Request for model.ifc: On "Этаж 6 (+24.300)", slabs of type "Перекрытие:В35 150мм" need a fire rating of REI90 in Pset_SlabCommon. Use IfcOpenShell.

First a look at what the model holds.

```python
import ifcopenshell
import ifcopenshell.util.element

model = ifcopenshell.open("model.ifc")
print(model.schema)
storey = next(s for s in model.by_type("IfcBuildingStorey") if s.Name == "Этаж 6 (+24.300)")
slabs = [e for e in ifcopenshell.util.element.get_decomposition(storey) if e.is_a("IfcSlab")]
seen = {}
for e in slabs:
    element_type = ifcopenshell.util.element.get_type(e)
    key = (element_type.Name if element_type != e and element_type else None, ifcopenshell.util.element.get_pset(e, "Pset_SlabCommon", "FireRating"))
    seen[key] = seen.get(key, 0) + 1
for (name, value), count in sorted(seen.items(), key=str):
    print(count, "x", name, "|", value)
```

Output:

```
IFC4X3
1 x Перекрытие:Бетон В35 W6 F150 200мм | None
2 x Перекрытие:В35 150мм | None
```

```python
import ifcopenshell
import ifcopenshell.api.pset
import ifcopenshell.util.element

model = ifcopenshell.open("model.ifc")

storey = next(s for s in model.by_type("IfcBuildingStorey") if s.Name == "Этаж 6 (+24.300)")
slabs = [e for e in ifcopenshell.util.element.get_decomposition(storey) if e.is_a("IfcSlab")]

count = 0
for e in slabs:
    element_type = ifcopenshell.util.element.get_type(e)
    if element_type in (None, e) or element_type.Name != "Перекрытие:В35 150мм":
        continue
    # add_pset returns the element's existing set when there is one.
    pset = ifcopenshell.api.pset.add_pset(model, product=e, name="Pset_SlabCommon")
    ifcopenshell.api.pset.edit_pset(model, pset=pset, properties={"FireRating": "REI90"})
    count += 1

print(count, "slabs updated")

model.write("model_v2.ifc")
```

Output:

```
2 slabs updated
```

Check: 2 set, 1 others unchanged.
